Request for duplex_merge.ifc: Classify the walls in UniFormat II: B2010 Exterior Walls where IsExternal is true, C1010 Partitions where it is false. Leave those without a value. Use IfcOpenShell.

First a look at what the model holds.

```python
import ifcopenshell
import ifcopenshell.util.element

model = ifcopenshell.open("duplex_merge.ifc")
print(model.schema)
print("classifications:", [c.Name for c in model.by_type("IfcClassification")])
values = [ifcopenshell.util.element.get_pset(e, "Pset_WallCommon", "IsExternal") for e in model.by_type("IfcWall")]
for value in (True, False, None):
    print("IsExternal", value, values.count(value))
```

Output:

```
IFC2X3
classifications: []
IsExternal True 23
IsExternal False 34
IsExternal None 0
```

```python
import ifcopenshell
import ifcopenshell.api.classification
import ifcopenshell.util.element

model = ifcopenshell.open("duplex_merge.ifc")

# IFC2X3 requires Source and Edition and has no link from the project to the system.
system = model.create_entity("IfcClassification", Source="ASTM", Edition="E1557", Name="UniFormat II")

walls = model.by_type("IfcWall")
external = {e: ifcopenshell.util.element.get_pset(e, "Pset_WallCommon", "IsExternal") for e in walls}
for flag, code, name in ((True, "B2010", "Exterior Walls"), (False, "C1010", "Partitions")):
    products = [e for e in walls if external[e] is flag]
    ifcopenshell.api.classification.add_reference(
        model, products=products, classification=system, identification=code, name=name
    )
    print(code, len(products))

model.write("duplex_merge_v2.ifc")
```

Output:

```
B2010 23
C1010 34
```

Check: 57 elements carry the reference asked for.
